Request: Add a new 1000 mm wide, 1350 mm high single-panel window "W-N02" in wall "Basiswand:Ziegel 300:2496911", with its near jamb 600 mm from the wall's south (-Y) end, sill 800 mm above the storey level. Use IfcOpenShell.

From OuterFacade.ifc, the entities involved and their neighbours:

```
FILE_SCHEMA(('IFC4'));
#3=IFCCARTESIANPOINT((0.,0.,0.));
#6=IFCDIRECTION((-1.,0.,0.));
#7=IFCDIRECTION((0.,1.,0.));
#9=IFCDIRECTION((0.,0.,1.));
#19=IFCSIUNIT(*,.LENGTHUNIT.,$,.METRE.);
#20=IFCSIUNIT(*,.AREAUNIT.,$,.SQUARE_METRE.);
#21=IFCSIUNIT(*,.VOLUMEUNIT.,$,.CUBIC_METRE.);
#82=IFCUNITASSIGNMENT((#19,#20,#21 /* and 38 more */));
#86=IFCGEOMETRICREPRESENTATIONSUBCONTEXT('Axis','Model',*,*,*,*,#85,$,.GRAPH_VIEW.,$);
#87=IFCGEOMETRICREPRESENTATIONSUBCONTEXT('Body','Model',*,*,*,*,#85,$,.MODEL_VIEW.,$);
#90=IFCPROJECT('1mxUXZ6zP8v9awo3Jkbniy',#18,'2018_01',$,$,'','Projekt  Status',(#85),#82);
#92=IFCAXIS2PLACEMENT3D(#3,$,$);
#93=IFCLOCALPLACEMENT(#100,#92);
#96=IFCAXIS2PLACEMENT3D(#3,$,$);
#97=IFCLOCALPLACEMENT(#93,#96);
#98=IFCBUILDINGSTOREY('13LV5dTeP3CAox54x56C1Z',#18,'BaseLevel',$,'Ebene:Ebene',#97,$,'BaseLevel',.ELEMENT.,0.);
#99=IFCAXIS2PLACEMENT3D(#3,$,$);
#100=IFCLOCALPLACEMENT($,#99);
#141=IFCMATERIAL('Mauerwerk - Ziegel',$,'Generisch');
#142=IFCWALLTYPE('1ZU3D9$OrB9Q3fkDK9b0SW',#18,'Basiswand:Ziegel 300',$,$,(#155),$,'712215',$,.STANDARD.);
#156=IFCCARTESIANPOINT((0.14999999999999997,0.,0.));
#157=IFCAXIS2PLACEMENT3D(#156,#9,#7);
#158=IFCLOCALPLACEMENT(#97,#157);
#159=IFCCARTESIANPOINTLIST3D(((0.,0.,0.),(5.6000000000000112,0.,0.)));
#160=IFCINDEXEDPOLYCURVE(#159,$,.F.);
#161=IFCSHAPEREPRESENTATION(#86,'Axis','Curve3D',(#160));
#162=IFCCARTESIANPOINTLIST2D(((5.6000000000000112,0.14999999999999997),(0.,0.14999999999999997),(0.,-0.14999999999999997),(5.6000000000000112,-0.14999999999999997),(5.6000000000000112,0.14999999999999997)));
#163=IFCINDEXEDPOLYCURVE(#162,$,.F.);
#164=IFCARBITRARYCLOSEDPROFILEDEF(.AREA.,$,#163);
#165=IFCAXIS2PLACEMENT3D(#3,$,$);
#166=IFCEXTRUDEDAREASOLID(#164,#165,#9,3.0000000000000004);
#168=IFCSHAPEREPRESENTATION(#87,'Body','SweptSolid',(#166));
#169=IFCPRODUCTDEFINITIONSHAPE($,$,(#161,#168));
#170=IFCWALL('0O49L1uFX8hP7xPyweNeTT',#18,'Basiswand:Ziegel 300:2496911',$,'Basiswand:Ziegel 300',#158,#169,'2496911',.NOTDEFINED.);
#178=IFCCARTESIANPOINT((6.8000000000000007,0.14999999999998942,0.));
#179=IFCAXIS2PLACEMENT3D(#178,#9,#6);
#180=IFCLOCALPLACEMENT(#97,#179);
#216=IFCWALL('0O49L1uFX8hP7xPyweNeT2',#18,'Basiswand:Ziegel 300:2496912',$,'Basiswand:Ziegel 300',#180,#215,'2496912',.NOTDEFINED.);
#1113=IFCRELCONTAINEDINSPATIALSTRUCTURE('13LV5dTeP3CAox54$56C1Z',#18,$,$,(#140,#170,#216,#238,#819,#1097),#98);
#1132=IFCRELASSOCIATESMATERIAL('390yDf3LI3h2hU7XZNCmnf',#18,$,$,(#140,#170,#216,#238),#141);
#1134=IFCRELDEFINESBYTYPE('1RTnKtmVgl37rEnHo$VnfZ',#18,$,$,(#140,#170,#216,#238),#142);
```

```python
import numpy as np
import ifcopenshell
import ifcopenshell.api.feature
import ifcopenshell.api.geometry
import ifcopenshell.api.root
import ifcopenshell.api.spatial
import ifcopenshell.geom
import ifcopenshell.util.element
import ifcopenshell.util.placement
import ifcopenshell.util.representation
import ifcopenshell.util.shape
import ifcopenshell.util.unit

model = ifcopenshell.open("OuterFacade.ifc")
unit_scale = ifcopenshell.util.unit.calculate_unit_scale(model)
settings = ifcopenshell.geom.settings()


def volume(element):
    """Net volume in cubic metres, openings subtracted."""
    shape = ifcopenshell.geom.create_shape(settings, element)
    return ifcopenshell.util.shape.get_volume(shape.geometry)


wall = model.by_id(170)
storey = ifcopenshell.util.element.get_container(wall, ifc_class="IfcBuildingStorey")
context = ifcopenshell.util.representation.get_context(model, "Model", "Body", "MODEL_VIEW")
before = volume(wall)

width, height, from_end, sill = 1, 1.35, 0.6, 0.8  # metres

# The wall runs along its own X axis, and the end named is its -X end.
wall_shape = ifcopenshell.geom.create_shape(settings, wall)
x, y, z = ifcopenshell.util.shape.get_vertices(wall_shape.geometry).T
start = x.min() + from_end
face, thickness = float(y.min()), float(y.max() - y.min())
wall_matrix = ifcopenshell.util.placement.get_local_placement(wall.ObjectPlacement)
level = ifcopenshell.util.placement.get_local_placement(storey.ObjectPlacement)[2, 3]


def in_wall(x, y):
    """Placement at x, y metres in the wall's axes, at sill height."""
    matrix = wall_matrix.copy()
    matrix[:, 3] = wall_matrix @ np.array([x / unit_scale, y / unit_scale, 0.0, 1.0])
    matrix[2, 3] = level + sill / unit_scale
    return matrix


# Opening: a box that overshoots both wall faces by 50 mm.
opening = ifcopenshell.api.root.create_entity(model, ifc_class="IfcOpeningElement", predefined_type="OPENING")
box = ifcopenshell.api.geometry.add_wall_representation(
    model, context=context, length=width, height=height, thickness=thickness + 0.1
)
ifcopenshell.api.geometry.assign_representation(model, product=opening, representation=box)
ifcopenshell.api.geometry.edit_object_placement(model, product=opening, matrix=in_wall(start, face - 0.05), is_si=False)
ifcopenshell.api.feature.add_feature(model, feature=opening, element=wall)

window = ifcopenshell.api.root.create_entity(model, ifc_class="IfcWindow", name="W-N02", predefined_type="WINDOW")
window.OverallWidth, window.OverallHeight = width / unit_scale, height / unit_scale
window.PartitioningType = "SINGLE_PANEL"
body = ifcopenshell.api.geometry.add_window_representation(
    model,
    context=context,
    overall_width=window.OverallWidth,
    overall_height=window.OverallHeight,
    partition_type="SINGLE_PANEL",
)
ifcopenshell.api.geometry.assign_representation(model, product=window, representation=body)
ifcopenshell.api.spatial.assign_container(model, products=[window], relating_structure=storey)
ifcopenshell.api.feature.add_filling(model, opening=opening, element=window)

# Centre the window in the wall's thickness.
ifcopenshell.api.geometry.edit_object_placement(model, product=window, matrix=in_wall(start, face), is_si=False)
window_shape = ifcopenshell.geom.create_shape(settings, window)
depth = ifcopenshell.util.shape.get_vertices(window_shape.geometry)[:, 1]
offset = face + thickness / 2 - (depth.min() + depth.max()) / 2
ifcopenshell.api.geometry.edit_object_placement(model, product=window, matrix=in_wall(start, offset), is_si=False)

after = volume(wall)

print(f"wall volume {before:.3f} -> {after:.3f} m3")

model.write("OuterFacade_v2.ifc")
```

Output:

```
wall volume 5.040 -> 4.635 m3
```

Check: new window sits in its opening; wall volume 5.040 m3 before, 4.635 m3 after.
